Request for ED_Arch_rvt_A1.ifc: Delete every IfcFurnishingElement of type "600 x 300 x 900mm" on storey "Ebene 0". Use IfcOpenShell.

First a look at what the model holds.

```python
import ifcopenshell
import ifcopenshell.util.element

model = ifcopenshell.open("ED_Arch_rvt_A1.ifc")
print(model.schema)
storey = next(s for s in model.by_type("IfcBuildingStorey") if s.Name == "Ebene 0")
furniture = [e for e in ifcopenshell.util.element.get_decomposition(storey) if e.is_a("IfcFurnishingElement")]
seen = {}
for e in furniture:
    element_type = ifcopenshell.util.element.get_type(e)
    name = element_type.Name if element_type not in (None, e) else None
    seen[name] = seen.get(name, 0) + 1
for name, count in sorted(seen.items(), key=str):
    print(count, "x", name)
```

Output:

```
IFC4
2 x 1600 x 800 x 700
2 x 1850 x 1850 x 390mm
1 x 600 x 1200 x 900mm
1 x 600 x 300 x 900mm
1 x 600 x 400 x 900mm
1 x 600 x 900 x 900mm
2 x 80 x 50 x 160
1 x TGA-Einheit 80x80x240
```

```python
import ifcopenshell
import ifcopenshell.api.root
import ifcopenshell.util.element

model = ifcopenshell.open("ED_Arch_rvt_A1.ifc")

storey = next(s for s in model.by_type("IfcBuildingStorey") if s.Name == "Ebene 0")
furniture = [e for e in ifcopenshell.util.element.get_decomposition(storey) if e.is_a("IfcFurnishingElement")]
targets = [e for e in furniture if (t := ifcopenshell.util.element.get_type(e)) not in (None, e) and t.Name == "600 x 300 x 900mm"]

for e in targets:
    ifcopenshell.api.root.remove_product(model, product=e)
print(len(targets), "removed")

model.write("ED_Arch_rvt_A1_edited.ifc")
```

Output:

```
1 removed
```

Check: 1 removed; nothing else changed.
